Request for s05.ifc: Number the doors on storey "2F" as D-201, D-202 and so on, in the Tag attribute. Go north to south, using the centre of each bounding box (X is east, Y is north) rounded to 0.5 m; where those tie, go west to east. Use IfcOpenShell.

First a look at what the model holds.

```python
import ifcopenshell
import ifcopenshell.util.element
import ifcopenshell.util.placement

model = ifcopenshell.open("s05.ifc")
print(model.schema)
storey = next(s for s in model.by_type("IfcBuildingStorey") if s.Name == "2F")
doors = [e for e in ifcopenshell.util.element.get_decomposition(storey) if e.is_a("IfcDoor")]
for e in sorted(doors, key=lambda e: e.id()):
    origin = ifcopenshell.util.placement.get_local_placement(e.ObjectPlacement)[:3, 3]
    print(e.id(), e.Tag, e.Name, origin.round(2) + 0.0, sep=" | ")
```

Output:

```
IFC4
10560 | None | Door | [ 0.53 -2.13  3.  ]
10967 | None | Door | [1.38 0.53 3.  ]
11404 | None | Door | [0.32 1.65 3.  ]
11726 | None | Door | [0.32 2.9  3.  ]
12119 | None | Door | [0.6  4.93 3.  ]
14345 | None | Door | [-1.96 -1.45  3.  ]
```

```python
import ifcopenshell
import ifcopenshell.geom
import ifcopenshell.util.element
import ifcopenshell.util.shape

model = ifcopenshell.open("s05.ifc")
settings = ifcopenshell.geom.settings()
settings.set("use-world-coords", True)


def centre(element):
    shape = ifcopenshell.geom.create_shape(settings, element)
    return ifcopenshell.util.shape.get_bbox_centroid(shape.geometry)


storey = next(s for s in model.by_type("IfcBuildingStorey") if s.Name == "2F")
doors = [e for e in ifcopenshell.util.element.get_decomposition(storey) if e.is_a("IfcDoor")]

# Insertion points can sit at a corner or the storey origin, so sort by the geometry (in metres).
centres = {e: centre(e) for e in doors}
doors.sort(key=lambda e: (-round(centres[e][1] / 0.5), centres[e][0]))

for i, e in enumerate(doors, start=1):
    number = f"D-2{i:02d}"
    e.Tag = number
    print(e.id(), number)

model.write("s05_rev.ifc")
```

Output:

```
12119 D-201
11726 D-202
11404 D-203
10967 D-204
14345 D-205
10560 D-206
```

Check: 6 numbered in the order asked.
